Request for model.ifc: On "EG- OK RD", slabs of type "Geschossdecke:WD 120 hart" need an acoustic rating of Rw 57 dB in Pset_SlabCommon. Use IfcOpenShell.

First a look at what the model holds.

```python
import ifcopenshell
import ifcopenshell.util.element

model = ifcopenshell.open("model.ifc")
print(model.schema)
storey = next(s for s in model.by_type("IfcBuildingStorey") if s.Name == "EG- OK RD")
slabs = [e for e in ifcopenshell.util.element.get_decomposition(storey) if e.is_a("IfcSlab")]
seen = {}
for e in slabs:
    element_type = ifcopenshell.util.element.get_type(e)
    key = (element_type.Name if element_type != e and element_type else None, ifcopenshell.util.element.get_pset(e, "Pset_SlabCommon", "AcousticRating"))
    seen[key] = seen.get(key, 0) + 1
for (name, value), count in sorted(seen.items(), key=str):
    print(count, "x", name, "|", value)
```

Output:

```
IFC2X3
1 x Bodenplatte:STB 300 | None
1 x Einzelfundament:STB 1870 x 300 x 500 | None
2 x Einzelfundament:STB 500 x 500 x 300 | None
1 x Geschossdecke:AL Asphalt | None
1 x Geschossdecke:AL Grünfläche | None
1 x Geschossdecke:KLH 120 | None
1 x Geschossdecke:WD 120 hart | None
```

```python
import ifcopenshell
import ifcopenshell.api.pset
import ifcopenshell.util.element

model = ifcopenshell.open("model.ifc")

storey = next(s for s in model.by_type("IfcBuildingStorey") if s.Name == "EG- OK RD")
slabs = [e for e in ifcopenshell.util.element.get_decomposition(storey) if e.is_a("IfcSlab")]

count = 0
for e in slabs:
    element_type = ifcopenshell.util.element.get_type(e)
    if element_type in (None, e) or element_type.Name != "Geschossdecke:WD 120 hart":
        continue
    # add_pset returns the element's existing set when there is one.
    pset = ifcopenshell.api.pset.add_pset(model, product=e, name="Pset_SlabCommon")
    ifcopenshell.api.pset.edit_pset(model, pset=pset, properties={"AcousticRating": "Rw 57 dB"})
    count += 1

print(count, "slabs updated")

model.write("model_v2.ifc")
```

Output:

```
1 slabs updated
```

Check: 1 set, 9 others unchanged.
